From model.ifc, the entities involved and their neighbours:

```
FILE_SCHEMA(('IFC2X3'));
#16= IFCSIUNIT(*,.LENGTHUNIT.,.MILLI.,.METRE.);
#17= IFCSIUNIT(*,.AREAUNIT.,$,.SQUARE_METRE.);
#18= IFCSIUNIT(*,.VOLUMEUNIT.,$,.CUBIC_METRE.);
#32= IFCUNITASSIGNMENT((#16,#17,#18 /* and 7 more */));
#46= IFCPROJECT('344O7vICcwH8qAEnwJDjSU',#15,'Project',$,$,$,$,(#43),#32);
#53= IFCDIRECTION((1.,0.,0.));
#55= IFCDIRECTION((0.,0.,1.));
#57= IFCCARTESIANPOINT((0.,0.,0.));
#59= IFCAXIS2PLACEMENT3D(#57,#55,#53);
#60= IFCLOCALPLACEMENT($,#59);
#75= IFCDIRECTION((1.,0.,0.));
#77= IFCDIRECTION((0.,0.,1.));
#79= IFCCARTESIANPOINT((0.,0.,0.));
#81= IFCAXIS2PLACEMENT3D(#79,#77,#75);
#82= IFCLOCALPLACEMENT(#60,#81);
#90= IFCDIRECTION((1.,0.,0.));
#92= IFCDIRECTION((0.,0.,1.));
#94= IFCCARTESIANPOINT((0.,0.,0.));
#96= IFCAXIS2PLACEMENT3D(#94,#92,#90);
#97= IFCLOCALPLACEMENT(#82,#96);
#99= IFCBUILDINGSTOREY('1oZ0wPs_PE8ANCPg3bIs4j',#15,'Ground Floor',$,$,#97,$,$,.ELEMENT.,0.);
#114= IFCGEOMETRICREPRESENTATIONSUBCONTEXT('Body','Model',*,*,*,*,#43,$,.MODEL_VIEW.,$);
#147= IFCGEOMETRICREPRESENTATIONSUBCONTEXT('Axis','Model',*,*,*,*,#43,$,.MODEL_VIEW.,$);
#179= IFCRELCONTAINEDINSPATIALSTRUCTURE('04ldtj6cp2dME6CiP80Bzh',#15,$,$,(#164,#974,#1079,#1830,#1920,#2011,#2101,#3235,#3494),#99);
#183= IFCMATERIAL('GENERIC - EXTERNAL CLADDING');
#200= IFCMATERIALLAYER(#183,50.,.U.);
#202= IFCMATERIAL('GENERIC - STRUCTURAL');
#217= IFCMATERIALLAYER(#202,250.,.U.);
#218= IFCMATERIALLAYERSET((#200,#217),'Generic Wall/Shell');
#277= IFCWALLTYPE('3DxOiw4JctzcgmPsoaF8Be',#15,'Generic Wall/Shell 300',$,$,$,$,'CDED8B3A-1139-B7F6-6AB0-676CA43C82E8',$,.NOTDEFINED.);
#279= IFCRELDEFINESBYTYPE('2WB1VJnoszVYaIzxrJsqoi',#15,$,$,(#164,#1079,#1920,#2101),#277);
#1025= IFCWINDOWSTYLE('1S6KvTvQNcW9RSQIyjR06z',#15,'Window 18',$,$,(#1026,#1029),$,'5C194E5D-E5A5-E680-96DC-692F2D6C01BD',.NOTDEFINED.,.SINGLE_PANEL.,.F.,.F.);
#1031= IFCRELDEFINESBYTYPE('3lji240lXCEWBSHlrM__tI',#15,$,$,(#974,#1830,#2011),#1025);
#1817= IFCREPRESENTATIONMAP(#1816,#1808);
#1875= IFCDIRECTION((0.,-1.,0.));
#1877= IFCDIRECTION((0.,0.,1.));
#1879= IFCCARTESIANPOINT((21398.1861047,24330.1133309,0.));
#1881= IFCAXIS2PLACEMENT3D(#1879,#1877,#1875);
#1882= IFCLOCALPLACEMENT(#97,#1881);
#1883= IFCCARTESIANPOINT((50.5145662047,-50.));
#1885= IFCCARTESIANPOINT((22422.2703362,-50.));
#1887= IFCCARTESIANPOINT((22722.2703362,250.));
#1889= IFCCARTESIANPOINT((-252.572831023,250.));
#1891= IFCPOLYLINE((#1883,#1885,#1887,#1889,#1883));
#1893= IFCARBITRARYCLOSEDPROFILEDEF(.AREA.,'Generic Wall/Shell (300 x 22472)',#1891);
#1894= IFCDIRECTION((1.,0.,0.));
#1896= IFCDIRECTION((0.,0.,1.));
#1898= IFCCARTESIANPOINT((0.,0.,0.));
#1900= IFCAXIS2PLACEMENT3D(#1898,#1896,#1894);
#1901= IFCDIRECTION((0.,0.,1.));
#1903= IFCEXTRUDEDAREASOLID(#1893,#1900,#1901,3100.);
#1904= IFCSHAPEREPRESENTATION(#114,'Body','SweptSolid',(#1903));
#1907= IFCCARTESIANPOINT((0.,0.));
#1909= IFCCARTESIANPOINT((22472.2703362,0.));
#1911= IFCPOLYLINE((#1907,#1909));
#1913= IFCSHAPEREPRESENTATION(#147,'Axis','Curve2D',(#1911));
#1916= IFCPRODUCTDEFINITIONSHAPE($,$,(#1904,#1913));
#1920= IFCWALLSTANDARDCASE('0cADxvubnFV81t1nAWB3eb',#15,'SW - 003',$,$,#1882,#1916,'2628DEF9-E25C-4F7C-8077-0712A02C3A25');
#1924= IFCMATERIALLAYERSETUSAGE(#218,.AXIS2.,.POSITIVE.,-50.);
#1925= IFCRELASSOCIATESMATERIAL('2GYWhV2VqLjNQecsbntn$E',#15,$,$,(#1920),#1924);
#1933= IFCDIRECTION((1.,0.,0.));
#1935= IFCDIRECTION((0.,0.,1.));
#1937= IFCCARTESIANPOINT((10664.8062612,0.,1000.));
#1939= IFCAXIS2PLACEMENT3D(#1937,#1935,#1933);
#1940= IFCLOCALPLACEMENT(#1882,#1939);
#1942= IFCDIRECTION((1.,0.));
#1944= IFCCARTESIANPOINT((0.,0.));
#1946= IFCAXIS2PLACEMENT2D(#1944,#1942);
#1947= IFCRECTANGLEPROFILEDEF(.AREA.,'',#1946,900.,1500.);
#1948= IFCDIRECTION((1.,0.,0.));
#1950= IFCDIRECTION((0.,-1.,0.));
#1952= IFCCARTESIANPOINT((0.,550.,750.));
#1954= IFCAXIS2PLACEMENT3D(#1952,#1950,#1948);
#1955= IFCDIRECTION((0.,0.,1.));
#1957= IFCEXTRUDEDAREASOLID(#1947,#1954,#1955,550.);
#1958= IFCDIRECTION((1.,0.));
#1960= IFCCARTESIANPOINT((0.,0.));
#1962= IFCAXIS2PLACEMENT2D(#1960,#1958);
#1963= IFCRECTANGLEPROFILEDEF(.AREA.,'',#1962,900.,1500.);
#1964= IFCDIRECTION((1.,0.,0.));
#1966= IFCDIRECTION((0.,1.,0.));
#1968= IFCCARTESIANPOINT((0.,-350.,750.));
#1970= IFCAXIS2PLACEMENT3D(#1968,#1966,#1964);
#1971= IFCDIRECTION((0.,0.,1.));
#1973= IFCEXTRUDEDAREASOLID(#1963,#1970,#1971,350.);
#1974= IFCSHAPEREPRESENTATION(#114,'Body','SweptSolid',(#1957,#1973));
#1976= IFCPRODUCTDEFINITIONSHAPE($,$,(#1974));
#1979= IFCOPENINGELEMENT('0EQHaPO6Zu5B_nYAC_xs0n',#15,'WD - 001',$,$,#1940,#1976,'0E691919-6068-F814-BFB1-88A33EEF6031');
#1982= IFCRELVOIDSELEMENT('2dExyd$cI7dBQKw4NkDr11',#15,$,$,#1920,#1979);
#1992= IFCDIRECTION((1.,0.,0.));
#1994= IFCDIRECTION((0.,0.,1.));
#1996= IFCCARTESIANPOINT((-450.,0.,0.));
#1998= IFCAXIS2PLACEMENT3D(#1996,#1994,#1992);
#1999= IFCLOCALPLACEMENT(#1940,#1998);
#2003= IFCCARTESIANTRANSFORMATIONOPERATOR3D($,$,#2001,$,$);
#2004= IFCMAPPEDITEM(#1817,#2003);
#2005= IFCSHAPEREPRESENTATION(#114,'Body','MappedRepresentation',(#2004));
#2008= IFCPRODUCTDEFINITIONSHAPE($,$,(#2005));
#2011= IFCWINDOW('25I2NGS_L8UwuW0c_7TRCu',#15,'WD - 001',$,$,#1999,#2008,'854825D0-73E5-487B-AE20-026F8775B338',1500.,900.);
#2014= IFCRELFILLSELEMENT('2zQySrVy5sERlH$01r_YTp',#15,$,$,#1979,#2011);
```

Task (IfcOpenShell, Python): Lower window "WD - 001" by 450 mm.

```python
import numpy as np
import ifcopenshell
import ifcopenshell.api.geometry
import ifcopenshell.util.placement
import ifcopenshell.util.unit

model = ifcopenshell.open("model.ifc")
unit_scale = ifcopenshell.util.unit.calculate_unit_scale(model)

window = model.by_guid("25I2NGS_L8UwuW0c_7TRCu")
opening = window.FillsVoids[0].RelatingOpeningElement
dz = -450.0

shift = np.array([0.0, 0.0, dz])
# The window is placed relative to its opening, so it follows when the opening moves.
matrix = ifcopenshell.util.placement.get_local_placement(opening.ObjectPlacement)
matrix[:3, 3] += shift
ifcopenshell.api.geometry.edit_object_placement(
    model, product=opening, matrix=matrix, is_si=False, should_transform_children=True
)

print(f"moved by {dz * unit_scale:+.3f} m")

model.write("model_rev.ifc")
```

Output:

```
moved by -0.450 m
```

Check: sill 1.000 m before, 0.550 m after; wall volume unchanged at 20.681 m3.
